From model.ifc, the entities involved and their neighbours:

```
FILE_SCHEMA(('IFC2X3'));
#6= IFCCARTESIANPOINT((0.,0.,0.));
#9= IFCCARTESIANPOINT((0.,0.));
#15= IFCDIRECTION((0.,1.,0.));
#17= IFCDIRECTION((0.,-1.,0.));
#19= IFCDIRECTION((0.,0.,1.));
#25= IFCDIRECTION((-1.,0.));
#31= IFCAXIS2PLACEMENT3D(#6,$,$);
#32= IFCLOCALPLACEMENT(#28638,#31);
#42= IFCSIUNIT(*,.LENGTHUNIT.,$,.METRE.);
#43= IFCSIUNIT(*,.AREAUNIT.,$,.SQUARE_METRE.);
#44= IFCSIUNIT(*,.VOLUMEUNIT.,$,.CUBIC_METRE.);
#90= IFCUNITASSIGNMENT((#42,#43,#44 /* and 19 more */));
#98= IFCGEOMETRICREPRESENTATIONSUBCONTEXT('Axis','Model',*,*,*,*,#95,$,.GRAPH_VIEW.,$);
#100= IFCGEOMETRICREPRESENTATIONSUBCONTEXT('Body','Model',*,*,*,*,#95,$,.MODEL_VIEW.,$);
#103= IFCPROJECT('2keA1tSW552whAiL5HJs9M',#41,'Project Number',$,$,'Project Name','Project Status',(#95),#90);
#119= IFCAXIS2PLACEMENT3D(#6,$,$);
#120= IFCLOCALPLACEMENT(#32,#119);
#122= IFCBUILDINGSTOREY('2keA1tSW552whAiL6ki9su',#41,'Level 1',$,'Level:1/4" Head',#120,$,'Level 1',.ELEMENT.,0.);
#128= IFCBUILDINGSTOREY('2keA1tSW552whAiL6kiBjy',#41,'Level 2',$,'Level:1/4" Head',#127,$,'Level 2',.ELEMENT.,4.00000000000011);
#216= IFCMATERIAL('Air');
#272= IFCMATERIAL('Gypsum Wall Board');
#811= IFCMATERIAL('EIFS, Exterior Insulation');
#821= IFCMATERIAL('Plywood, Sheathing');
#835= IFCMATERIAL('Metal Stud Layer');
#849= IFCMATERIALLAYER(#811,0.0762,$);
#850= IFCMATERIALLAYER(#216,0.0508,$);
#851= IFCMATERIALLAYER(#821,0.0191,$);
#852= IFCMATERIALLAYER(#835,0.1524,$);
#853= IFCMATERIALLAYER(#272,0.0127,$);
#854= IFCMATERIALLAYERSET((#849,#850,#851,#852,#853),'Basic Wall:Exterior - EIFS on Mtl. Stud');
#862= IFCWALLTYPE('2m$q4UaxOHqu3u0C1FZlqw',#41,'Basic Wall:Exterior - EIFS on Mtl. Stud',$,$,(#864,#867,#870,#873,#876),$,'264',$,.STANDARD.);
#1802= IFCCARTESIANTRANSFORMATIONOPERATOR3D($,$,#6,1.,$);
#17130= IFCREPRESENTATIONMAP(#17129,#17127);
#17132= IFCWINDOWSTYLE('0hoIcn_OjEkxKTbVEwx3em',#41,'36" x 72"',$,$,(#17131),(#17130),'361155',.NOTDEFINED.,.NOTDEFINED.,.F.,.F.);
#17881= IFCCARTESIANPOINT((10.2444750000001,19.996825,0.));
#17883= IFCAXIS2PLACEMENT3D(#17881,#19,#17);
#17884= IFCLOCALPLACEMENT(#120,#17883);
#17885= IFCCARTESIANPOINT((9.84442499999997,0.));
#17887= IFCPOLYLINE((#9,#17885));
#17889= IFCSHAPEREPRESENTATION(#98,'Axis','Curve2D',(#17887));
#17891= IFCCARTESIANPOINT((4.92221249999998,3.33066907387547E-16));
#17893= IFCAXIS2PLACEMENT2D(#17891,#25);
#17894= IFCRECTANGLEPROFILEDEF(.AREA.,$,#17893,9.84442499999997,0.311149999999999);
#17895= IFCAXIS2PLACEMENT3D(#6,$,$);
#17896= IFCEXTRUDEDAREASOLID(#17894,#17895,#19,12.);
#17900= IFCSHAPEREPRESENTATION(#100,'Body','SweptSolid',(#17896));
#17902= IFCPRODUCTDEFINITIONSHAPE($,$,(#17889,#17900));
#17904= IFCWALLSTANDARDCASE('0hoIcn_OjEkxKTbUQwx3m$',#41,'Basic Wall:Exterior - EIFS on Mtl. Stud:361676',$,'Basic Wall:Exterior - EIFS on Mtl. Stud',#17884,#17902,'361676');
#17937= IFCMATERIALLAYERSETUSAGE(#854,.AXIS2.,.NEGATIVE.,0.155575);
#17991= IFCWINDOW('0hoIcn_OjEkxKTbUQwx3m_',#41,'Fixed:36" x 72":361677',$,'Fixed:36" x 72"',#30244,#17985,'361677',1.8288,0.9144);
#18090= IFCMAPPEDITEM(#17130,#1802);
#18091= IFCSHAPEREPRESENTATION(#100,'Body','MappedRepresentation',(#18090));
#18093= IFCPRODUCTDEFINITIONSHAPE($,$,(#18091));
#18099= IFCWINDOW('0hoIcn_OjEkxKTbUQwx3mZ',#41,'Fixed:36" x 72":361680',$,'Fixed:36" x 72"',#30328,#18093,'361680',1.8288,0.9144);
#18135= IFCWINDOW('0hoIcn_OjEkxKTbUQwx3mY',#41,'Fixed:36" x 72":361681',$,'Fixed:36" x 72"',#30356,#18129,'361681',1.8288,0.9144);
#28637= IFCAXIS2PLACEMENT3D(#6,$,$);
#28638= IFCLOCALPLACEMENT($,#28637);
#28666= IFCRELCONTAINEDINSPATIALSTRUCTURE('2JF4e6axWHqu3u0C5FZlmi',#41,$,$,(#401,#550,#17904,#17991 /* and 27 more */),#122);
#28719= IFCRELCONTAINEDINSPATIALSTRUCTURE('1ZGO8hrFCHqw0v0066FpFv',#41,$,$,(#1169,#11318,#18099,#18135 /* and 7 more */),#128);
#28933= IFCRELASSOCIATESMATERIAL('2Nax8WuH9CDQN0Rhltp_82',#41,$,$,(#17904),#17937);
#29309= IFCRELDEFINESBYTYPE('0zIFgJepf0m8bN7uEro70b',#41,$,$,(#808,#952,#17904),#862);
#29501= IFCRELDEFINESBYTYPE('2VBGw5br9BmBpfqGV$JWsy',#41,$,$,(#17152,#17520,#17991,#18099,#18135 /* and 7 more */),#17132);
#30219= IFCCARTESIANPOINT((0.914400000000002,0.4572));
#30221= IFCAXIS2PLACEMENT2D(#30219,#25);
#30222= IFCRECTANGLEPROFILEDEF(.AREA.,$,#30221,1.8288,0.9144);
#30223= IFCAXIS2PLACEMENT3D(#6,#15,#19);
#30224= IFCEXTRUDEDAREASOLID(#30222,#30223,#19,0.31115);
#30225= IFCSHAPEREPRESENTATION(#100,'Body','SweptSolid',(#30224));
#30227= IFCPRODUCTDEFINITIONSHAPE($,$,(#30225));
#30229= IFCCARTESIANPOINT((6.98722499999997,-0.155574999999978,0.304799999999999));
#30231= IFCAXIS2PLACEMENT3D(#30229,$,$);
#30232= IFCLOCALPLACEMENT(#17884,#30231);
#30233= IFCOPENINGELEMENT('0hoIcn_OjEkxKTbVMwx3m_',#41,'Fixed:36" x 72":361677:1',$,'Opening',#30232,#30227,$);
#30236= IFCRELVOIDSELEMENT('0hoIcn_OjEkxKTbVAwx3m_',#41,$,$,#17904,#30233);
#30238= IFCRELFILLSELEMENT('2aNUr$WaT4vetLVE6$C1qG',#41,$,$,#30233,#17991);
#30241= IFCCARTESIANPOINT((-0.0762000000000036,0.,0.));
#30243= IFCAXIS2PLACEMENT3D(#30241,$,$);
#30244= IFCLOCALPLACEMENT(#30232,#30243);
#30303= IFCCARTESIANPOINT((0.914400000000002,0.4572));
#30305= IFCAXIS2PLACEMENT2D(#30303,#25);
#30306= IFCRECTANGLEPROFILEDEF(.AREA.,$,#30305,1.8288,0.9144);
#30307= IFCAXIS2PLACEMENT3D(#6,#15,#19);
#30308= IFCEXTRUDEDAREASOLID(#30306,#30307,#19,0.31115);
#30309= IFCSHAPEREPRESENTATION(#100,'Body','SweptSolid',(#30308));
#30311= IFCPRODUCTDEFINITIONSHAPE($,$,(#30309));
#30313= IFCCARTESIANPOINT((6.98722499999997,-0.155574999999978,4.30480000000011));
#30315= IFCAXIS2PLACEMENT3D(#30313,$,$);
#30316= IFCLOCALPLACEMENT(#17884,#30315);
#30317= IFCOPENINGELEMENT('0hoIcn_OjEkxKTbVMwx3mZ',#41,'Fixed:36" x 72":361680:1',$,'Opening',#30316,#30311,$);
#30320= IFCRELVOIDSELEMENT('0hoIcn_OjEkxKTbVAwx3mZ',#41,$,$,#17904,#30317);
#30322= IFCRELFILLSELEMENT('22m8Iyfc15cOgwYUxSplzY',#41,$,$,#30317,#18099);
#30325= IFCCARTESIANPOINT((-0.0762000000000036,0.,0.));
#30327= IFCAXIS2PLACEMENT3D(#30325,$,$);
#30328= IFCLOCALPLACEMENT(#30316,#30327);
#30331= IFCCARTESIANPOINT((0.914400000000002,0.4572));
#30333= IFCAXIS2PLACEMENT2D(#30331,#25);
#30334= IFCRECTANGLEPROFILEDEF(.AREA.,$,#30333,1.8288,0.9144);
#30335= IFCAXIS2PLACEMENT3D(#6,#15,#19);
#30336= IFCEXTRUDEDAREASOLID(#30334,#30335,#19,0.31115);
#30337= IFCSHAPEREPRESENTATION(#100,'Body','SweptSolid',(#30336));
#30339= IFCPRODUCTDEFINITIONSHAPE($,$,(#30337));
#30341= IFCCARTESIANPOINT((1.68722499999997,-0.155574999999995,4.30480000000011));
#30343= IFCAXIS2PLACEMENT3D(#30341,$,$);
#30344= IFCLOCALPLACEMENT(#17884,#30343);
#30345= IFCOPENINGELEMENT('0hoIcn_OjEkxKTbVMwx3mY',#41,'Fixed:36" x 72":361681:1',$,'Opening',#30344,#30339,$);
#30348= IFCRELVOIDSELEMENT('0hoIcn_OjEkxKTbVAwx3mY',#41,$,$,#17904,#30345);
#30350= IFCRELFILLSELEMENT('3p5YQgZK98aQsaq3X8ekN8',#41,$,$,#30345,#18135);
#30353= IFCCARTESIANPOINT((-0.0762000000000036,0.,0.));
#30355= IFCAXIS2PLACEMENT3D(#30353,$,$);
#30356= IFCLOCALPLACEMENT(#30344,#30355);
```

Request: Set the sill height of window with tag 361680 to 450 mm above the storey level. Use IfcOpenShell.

```python
import numpy as np
import ifcopenshell
import ifcopenshell.api.geometry
import ifcopenshell.geom
import ifcopenshell.util.element
import ifcopenshell.util.placement
import ifcopenshell.util.shape
import ifcopenshell.util.unit

model = ifcopenshell.open("model.ifc")
unit_scale = ifcopenshell.util.unit.calculate_unit_scale(model)

window = model.by_guid("0hoIcn_OjEkxKTbUQwx3mZ")
opening = window.FillsVoids[0].RelatingOpeningElement
storey = ifcopenshell.util.element.get_container(window, ifc_class="IfcBuildingStorey")
level = ifcopenshell.util.placement.get_local_placement(storey.ObjectPlacement)[2, 3]

# The opening's origin need not be at the sill, so measure its lowest point.
shape = ifcopenshell.geom.create_shape(ifcopenshell.geom.settings(), opening)
bottom = ifcopenshell.util.shape.get_shape_bottom_elevation(shape, shape.geometry) / unit_scale
dz = level + 0.45 / unit_scale - bottom

shift = np.array([0.0, 0.0, dz])
# The window is placed relative to its opening, so it follows when the opening moves.
matrix = ifcopenshell.util.placement.get_local_placement(opening.ObjectPlacement)
matrix[:3, 3] += shift
ifcopenshell.api.geometry.edit_object_placement(
    model, product=opening, matrix=matrix, is_si=False, should_transform_children=True
)

print(f"moved by {dz * unit_scale:+.3f} m")

model.write("model_v2.ifc")
```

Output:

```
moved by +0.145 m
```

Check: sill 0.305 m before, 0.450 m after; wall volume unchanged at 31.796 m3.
